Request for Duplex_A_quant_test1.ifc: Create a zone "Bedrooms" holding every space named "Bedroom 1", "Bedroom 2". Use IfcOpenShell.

First a look at what the model holds.

```python
import ifcopenshell

model = ifcopenshell.open("Duplex_A_quant_test1.ifc")
print(model.schema)
seen = {}
for space in model.by_type("IfcSpace"):
    seen[space.LongName] = seen.get(space.LongName, 0) + 1
for name, count in sorted(seen.items(), key=str):
    print(count, "x", name)
print("zones:", [z.Name for z in model.by_type("IfcZone")][:20])
```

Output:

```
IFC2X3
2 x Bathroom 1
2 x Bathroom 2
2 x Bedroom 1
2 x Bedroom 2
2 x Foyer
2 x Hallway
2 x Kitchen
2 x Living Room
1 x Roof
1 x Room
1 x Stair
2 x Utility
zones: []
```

```python
import ifcopenshell
import ifcopenshell.api.group
import ifcopenshell.api.root

model = ifcopenshell.open("Duplex_A_quant_test1.ifc")

names = {"Bedroom 1", "Bedroom 2"}
spaces = [s for s in model.by_type("IfcSpace") if s.LongName in names]

zone = ifcopenshell.api.root.create_entity(model, ifc_class="IfcZone", name="Bedrooms")
ifcopenshell.api.group.assign_group(model, products=spaces, group=zone)
print(len(spaces), "spaces in", zone.Name)

model.write("Duplex_A_quant_test1_v2.ifc")
```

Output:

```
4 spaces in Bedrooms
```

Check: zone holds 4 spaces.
